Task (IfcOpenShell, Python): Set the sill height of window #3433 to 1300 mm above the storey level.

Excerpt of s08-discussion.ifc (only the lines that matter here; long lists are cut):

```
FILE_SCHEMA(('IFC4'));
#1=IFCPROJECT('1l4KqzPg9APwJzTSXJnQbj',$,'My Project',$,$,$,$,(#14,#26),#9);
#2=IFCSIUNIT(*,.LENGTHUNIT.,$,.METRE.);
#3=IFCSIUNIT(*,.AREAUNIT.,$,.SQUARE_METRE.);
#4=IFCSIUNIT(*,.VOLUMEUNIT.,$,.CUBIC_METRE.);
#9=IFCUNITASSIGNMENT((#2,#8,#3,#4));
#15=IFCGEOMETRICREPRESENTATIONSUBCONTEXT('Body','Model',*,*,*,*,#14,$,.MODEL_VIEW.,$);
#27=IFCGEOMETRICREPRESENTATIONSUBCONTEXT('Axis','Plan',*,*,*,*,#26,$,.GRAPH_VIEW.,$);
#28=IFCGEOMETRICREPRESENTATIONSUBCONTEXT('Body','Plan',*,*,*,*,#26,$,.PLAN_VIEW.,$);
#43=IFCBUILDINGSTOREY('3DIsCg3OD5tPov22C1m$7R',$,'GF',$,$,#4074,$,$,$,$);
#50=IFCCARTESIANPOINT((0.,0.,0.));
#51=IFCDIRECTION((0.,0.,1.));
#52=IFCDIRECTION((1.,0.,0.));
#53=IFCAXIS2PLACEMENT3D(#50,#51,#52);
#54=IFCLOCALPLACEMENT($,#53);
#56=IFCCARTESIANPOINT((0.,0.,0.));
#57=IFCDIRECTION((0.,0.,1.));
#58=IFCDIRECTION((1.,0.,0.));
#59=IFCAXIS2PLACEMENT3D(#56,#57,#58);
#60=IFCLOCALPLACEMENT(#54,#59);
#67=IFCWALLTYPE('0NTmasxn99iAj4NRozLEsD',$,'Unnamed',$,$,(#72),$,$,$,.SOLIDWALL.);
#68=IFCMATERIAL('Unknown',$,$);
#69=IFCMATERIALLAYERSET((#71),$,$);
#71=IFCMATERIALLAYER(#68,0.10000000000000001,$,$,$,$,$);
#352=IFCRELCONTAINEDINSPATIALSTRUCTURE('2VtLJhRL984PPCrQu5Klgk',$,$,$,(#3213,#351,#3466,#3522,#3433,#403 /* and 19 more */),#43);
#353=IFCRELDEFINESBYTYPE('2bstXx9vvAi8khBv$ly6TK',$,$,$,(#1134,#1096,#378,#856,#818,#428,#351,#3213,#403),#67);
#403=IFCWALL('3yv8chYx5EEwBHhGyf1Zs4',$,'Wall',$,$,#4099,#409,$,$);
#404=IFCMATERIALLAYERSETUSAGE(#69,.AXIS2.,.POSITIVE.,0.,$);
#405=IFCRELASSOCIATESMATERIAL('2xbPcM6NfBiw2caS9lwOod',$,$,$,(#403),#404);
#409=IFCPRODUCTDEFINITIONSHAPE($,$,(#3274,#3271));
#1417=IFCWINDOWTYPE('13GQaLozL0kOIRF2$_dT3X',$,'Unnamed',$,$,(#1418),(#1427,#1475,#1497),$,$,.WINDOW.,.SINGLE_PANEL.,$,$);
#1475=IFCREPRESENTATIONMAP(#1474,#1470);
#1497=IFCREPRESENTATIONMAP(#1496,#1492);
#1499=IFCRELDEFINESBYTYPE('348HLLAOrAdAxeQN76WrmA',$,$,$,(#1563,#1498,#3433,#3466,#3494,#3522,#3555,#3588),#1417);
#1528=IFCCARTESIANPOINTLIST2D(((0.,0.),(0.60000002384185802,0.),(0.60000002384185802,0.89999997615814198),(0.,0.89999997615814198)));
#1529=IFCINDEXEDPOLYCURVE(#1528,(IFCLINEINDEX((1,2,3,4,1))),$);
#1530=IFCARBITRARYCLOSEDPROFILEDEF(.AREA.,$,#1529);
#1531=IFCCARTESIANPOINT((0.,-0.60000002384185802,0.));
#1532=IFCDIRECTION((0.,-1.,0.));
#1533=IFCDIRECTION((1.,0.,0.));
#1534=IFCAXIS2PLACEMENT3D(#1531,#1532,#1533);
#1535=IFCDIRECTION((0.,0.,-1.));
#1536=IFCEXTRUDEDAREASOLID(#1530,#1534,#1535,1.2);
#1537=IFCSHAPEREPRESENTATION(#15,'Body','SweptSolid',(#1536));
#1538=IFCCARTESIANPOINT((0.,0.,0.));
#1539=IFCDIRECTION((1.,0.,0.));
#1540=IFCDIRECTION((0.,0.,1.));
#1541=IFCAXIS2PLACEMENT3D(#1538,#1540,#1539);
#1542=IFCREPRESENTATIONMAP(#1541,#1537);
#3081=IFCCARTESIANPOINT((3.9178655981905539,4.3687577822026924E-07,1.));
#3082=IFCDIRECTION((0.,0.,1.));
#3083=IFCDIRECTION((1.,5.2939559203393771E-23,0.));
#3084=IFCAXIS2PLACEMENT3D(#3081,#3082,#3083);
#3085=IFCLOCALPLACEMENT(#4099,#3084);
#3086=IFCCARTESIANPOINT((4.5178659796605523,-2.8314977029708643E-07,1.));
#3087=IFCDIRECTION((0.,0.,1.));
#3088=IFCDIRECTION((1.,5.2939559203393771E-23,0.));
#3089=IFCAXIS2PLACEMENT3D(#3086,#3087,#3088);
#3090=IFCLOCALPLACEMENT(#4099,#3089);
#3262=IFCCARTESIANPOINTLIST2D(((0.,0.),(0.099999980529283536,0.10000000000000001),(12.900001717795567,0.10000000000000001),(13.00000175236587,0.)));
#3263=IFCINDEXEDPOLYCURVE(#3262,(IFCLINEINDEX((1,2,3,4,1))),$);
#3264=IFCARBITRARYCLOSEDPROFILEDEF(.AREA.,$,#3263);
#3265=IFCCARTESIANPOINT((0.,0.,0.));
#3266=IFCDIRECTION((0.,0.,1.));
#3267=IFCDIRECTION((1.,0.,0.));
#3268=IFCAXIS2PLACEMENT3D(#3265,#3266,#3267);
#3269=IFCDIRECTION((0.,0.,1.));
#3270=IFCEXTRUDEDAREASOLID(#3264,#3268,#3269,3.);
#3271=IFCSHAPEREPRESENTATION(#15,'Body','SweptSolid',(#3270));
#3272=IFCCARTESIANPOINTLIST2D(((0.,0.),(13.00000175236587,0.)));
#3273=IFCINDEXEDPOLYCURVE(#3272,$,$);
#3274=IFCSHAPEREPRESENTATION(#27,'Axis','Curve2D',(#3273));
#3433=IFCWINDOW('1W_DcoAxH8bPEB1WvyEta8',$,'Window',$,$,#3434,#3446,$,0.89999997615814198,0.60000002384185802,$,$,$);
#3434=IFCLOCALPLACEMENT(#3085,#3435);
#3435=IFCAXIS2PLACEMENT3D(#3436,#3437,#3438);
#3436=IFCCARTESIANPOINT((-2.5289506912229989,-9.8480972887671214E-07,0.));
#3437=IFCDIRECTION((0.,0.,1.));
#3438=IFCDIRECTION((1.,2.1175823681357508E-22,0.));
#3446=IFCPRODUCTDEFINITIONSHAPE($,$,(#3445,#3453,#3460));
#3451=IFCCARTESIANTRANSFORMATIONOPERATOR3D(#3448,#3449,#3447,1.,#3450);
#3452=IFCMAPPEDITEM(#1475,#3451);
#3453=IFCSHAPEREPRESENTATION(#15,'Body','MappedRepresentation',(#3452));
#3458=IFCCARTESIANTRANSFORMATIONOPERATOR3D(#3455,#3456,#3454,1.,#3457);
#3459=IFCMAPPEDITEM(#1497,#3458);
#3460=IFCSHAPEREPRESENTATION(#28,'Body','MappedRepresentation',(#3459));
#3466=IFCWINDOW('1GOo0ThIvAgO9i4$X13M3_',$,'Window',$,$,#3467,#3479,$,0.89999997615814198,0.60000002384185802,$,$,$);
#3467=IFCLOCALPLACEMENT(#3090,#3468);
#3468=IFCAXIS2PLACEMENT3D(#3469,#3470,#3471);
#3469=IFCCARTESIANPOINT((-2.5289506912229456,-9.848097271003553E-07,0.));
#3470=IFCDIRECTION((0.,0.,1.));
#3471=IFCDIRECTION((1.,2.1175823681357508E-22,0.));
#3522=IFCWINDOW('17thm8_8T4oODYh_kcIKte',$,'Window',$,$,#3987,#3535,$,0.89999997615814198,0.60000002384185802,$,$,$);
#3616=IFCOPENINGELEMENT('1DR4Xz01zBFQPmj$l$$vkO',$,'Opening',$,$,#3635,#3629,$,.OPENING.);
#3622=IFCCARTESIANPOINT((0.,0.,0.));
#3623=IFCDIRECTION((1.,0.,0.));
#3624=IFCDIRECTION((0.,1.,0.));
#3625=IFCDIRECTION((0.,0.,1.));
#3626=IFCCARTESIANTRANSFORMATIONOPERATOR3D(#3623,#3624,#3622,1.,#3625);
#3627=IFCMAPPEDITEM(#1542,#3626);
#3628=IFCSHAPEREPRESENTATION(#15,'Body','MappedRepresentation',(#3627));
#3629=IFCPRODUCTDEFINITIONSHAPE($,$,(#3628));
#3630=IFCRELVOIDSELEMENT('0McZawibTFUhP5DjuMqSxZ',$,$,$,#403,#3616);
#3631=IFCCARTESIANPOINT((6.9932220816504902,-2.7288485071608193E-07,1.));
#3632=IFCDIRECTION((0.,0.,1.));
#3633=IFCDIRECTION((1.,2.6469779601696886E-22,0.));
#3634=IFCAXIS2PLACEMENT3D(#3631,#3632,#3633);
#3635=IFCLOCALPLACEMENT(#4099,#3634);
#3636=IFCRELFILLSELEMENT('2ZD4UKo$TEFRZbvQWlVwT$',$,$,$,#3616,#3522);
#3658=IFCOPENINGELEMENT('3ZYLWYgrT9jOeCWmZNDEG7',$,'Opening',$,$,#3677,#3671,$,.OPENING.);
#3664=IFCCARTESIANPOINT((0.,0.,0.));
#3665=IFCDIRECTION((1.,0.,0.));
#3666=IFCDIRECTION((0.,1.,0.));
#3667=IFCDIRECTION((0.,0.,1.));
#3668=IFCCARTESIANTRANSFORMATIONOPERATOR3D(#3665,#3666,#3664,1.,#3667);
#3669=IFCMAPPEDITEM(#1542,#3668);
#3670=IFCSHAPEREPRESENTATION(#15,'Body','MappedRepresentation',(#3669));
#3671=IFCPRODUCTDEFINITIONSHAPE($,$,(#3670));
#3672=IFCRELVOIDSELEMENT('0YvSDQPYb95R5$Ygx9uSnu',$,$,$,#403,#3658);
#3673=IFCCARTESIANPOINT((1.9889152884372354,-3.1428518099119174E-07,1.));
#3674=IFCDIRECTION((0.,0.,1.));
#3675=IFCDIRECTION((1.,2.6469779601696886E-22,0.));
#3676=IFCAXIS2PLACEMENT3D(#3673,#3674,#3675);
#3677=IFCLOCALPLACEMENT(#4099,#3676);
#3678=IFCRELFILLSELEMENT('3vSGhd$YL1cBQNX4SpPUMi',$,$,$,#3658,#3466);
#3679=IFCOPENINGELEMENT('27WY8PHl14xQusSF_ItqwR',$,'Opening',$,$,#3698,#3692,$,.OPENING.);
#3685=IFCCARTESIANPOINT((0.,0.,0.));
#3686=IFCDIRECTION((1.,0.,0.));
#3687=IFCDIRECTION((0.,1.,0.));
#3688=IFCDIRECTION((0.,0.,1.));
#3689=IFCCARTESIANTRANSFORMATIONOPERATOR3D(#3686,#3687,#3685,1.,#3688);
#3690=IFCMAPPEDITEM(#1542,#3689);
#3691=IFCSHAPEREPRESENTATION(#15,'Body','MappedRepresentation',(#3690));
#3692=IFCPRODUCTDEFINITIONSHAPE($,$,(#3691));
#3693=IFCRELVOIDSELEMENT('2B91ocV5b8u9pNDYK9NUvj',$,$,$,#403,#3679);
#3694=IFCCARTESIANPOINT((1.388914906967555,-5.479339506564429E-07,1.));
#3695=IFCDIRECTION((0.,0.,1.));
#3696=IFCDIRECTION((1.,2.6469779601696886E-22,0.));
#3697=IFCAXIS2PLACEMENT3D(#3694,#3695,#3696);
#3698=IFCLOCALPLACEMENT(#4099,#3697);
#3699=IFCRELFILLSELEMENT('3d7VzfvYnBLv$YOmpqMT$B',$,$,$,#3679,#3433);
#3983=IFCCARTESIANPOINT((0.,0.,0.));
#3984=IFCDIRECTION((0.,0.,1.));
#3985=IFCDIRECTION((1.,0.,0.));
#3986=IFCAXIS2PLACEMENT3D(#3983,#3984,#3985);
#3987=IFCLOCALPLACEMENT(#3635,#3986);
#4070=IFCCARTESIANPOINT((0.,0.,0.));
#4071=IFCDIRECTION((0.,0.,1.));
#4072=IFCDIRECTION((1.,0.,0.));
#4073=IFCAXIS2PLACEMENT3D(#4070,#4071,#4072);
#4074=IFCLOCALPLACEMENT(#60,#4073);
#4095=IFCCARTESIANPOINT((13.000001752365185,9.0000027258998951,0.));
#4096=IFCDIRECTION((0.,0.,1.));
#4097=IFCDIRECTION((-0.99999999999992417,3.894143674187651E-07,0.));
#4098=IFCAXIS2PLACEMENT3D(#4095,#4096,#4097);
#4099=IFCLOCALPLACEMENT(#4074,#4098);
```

```python
import numpy as np
import ifcopenshell
import ifcopenshell.api.geometry
import ifcopenshell.geom
import ifcopenshell.util.element
import ifcopenshell.util.placement
import ifcopenshell.util.shape
import ifcopenshell.util.unit

model = ifcopenshell.open("s08-discussion.ifc")
unit_scale = ifcopenshell.util.unit.calculate_unit_scale(model)

window = model.by_guid("1W_DcoAxH8bPEB1WvyEta8")
opening = window.FillsVoids[0].RelatingOpeningElement
storey = ifcopenshell.util.element.get_container(window, ifc_class="IfcBuildingStorey")
level = ifcopenshell.util.placement.get_local_placement(storey.ObjectPlacement)[2, 3]

# The opening's origin need not be at the sill, so measure its lowest point.
shape = ifcopenshell.geom.create_shape(ifcopenshell.geom.settings(), opening)
bottom = ifcopenshell.util.shape.get_shape_bottom_elevation(shape, shape.geometry) / unit_scale
dz = level + 1.3 / unit_scale - bottom

shift = np.array([0.0, 0.0, dz])
# The window is not placed relative to its opening, so move both.
for product in (opening, window):
    matrix = ifcopenshell.util.placement.get_local_placement(product.ObjectPlacement)
    matrix[:3, 3] += shift
    ifcopenshell.api.geometry.edit_object_placement(model, product=product, matrix=matrix, is_si=False)

print(f"moved by {dz * unit_scale:+.3f} m")

model.write("s08-discussion_rev.ifc")
```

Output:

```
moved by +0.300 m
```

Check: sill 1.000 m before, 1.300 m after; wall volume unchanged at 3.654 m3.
